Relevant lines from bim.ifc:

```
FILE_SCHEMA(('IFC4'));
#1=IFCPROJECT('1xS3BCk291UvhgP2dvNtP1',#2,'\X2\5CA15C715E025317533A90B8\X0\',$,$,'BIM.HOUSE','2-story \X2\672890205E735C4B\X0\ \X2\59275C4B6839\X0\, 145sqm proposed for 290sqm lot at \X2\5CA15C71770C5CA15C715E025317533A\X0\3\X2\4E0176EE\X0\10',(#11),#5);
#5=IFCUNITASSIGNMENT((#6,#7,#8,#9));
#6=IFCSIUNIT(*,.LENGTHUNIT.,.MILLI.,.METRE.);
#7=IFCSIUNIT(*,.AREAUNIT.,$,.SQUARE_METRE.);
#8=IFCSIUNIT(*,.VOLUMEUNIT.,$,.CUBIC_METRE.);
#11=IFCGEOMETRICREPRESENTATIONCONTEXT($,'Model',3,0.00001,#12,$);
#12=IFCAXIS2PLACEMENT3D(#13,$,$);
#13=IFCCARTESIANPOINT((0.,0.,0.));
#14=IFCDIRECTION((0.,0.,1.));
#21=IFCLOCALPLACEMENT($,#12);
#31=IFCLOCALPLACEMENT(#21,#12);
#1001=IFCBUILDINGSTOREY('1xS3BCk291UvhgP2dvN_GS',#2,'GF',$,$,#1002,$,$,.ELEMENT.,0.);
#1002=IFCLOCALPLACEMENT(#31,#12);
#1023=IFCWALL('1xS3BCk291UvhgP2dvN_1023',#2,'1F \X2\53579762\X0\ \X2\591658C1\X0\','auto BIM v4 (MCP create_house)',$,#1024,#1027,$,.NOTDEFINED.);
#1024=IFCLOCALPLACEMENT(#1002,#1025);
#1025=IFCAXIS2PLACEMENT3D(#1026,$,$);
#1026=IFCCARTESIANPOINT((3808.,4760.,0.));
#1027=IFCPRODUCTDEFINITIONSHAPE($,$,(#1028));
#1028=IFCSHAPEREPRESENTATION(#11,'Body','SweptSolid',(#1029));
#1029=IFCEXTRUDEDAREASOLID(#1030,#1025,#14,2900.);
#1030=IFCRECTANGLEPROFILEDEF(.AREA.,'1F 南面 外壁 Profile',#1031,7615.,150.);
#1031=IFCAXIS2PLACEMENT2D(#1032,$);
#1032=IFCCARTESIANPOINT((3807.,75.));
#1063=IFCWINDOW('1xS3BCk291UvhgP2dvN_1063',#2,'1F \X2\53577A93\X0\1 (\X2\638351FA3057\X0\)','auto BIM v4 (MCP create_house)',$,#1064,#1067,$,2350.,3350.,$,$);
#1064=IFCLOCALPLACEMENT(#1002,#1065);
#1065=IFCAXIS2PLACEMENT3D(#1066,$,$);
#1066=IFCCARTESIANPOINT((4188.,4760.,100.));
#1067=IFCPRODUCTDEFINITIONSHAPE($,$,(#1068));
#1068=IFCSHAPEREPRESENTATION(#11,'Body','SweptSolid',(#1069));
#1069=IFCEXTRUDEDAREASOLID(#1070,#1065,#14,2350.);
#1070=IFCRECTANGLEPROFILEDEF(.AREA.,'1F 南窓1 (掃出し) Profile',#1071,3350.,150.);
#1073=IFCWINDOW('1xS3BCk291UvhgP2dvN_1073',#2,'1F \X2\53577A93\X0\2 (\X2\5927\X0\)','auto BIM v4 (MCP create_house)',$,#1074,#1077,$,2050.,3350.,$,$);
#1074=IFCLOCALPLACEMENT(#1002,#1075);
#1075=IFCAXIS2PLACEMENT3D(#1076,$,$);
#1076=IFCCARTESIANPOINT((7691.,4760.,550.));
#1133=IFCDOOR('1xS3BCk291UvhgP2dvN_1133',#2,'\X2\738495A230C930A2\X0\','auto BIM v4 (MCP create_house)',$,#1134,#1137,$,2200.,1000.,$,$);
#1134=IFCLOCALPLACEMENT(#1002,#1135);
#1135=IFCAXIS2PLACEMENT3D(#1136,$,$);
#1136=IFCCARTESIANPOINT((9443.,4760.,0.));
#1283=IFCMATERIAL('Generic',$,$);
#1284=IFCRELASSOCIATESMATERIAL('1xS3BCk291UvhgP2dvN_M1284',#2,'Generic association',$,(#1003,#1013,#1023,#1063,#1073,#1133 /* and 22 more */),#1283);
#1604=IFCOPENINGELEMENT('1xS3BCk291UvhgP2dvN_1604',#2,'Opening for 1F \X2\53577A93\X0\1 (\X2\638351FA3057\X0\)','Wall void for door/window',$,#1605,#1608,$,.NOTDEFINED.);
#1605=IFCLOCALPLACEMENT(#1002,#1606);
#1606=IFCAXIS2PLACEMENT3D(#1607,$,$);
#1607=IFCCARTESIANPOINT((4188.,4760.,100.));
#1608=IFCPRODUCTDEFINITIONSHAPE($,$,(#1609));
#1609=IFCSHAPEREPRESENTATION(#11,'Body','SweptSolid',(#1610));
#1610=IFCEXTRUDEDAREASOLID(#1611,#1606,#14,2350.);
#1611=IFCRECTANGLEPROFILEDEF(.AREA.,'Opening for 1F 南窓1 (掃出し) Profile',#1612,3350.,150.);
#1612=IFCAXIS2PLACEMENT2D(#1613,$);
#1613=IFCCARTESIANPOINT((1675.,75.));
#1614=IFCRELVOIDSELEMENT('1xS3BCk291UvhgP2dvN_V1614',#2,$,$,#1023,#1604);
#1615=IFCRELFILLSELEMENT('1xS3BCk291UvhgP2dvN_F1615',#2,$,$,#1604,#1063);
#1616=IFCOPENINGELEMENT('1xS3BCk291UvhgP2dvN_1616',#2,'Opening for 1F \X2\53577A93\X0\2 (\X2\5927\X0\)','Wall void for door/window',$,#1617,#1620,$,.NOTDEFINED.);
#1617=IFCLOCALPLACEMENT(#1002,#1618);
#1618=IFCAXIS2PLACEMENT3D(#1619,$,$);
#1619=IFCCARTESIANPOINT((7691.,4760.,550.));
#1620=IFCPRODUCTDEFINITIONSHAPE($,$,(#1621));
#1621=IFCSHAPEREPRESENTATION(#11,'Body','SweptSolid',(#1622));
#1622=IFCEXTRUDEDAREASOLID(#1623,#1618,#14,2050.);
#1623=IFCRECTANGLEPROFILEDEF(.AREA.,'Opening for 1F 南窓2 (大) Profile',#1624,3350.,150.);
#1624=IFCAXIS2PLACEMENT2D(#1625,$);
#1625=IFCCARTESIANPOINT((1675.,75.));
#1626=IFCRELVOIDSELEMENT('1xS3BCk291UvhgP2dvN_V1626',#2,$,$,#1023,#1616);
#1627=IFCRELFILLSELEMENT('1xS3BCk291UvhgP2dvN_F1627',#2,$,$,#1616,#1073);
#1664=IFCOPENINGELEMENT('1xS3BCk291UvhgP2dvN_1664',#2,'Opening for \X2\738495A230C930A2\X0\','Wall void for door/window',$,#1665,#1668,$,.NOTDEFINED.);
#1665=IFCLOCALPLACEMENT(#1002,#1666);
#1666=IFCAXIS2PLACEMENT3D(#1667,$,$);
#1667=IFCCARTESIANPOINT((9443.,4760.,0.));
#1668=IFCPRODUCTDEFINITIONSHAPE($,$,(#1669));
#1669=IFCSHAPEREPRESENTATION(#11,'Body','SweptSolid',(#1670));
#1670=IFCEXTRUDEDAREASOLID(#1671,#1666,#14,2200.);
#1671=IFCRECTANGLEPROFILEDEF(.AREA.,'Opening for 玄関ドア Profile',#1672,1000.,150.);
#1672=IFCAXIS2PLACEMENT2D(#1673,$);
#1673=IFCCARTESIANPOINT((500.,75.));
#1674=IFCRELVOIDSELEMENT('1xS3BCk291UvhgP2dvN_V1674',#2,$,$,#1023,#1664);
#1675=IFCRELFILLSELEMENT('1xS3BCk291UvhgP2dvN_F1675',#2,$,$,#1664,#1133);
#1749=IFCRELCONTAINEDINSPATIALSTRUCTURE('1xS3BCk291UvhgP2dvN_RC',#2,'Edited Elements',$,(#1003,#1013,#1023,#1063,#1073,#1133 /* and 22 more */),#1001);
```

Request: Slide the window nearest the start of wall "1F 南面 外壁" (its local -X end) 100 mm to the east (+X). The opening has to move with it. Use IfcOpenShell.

```python
import ifcopenshell
import ifcopenshell.api.geometry
import ifcopenshell.util.placement
import ifcopenshell.util.unit

model = ifcopenshell.open("bim.ifc")
unit_scale = ifcopenshell.util.unit.calculate_unit_scale(model)

window = model.by_guid("1xS3BCk291UvhgP2dvN_1063")
opening = window.FillsVoids[0].RelatingOpeningElement
wall = opening.VoidsElements[0].RelatingBuildingElement

wall_matrix = ifcopenshell.util.placement.get_local_placement(wall.ObjectPlacement)
shift = wall_matrix[:3, 0] * 0.1 / unit_scale
before = ifcopenshell.util.placement.get_local_placement(window.ObjectPlacement)[:3, 3].copy()

# The window is not placed relative to its opening, so move both.
for product in (opening, window):
    matrix = ifcopenshell.util.placement.get_local_placement(product.ObjectPlacement)
    matrix[:3, 3] += shift
    ifcopenshell.api.geometry.edit_object_placement(model, product=product, matrix=matrix, is_si=False)

after = ifcopenshell.util.placement.get_local_placement(window.ObjectPlacement)[:3, 3]
print("window moved by", (after - before).round(3) + 0.0)

model.write("bim_edited.ifc")
```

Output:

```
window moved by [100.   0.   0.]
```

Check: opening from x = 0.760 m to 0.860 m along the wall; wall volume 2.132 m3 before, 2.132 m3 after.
